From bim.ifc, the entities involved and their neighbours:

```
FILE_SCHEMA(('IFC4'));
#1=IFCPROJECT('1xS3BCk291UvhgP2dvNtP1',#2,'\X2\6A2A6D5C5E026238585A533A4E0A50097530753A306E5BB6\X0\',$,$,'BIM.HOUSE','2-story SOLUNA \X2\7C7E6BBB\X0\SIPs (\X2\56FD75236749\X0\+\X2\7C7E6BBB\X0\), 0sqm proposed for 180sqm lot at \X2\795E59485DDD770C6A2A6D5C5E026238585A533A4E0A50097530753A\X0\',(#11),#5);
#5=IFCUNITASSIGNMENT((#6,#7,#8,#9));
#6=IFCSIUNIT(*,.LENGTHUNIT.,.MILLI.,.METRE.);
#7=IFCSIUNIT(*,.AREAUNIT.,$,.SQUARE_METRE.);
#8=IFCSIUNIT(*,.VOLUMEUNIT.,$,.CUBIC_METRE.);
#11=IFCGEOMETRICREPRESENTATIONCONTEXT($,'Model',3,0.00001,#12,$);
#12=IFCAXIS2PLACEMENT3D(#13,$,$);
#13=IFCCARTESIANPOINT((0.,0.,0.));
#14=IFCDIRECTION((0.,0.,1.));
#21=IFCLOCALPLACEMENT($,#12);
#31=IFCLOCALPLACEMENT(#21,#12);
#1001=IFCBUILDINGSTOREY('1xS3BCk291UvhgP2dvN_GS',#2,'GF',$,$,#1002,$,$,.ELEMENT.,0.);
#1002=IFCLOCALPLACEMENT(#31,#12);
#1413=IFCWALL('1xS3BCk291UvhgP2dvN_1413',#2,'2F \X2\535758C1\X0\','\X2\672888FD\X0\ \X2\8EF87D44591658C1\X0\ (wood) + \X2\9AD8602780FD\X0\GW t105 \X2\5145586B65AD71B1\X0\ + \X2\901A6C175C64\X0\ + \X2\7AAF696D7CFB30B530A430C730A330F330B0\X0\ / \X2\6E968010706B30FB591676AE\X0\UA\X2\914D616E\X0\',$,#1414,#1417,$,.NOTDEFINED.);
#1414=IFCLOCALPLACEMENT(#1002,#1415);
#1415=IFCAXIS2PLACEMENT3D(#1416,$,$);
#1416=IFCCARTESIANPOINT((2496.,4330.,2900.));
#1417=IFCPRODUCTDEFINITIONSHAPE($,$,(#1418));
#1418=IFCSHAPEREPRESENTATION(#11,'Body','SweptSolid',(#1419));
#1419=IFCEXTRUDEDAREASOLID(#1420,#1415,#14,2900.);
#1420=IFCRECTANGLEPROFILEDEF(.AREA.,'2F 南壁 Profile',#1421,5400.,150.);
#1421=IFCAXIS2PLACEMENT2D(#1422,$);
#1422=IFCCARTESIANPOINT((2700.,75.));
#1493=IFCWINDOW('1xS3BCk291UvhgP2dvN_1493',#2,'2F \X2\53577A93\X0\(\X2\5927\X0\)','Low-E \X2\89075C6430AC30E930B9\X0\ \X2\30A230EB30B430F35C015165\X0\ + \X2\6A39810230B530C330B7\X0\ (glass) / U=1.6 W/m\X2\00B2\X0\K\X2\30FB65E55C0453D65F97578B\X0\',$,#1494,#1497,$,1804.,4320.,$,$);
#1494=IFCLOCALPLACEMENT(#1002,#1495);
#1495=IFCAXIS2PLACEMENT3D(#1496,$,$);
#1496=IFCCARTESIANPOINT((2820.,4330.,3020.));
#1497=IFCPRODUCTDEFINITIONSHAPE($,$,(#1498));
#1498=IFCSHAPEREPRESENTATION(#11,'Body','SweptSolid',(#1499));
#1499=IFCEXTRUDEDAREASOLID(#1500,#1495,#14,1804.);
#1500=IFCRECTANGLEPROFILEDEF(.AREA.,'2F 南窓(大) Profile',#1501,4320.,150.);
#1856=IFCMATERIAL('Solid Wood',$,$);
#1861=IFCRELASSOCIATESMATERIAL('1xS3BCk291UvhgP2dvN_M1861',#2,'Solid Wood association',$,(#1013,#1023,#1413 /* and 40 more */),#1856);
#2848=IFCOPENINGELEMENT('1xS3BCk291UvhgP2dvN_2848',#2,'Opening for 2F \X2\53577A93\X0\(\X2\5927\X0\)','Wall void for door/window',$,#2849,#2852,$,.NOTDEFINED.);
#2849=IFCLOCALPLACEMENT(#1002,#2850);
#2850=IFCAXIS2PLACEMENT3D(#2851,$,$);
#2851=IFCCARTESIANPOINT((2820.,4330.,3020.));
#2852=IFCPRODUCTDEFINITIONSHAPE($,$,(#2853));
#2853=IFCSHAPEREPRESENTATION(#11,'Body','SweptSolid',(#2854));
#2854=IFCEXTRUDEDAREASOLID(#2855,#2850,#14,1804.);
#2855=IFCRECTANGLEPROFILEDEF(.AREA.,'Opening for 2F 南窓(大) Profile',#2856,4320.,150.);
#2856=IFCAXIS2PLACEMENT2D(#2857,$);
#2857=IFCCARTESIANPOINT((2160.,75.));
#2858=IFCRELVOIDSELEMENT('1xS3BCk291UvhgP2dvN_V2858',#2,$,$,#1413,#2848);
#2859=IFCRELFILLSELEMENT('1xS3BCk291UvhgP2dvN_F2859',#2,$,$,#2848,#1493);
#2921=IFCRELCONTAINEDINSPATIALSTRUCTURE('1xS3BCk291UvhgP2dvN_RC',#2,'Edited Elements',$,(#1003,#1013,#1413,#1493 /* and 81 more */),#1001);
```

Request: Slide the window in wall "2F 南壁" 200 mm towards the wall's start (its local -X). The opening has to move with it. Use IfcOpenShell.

```python
import ifcopenshell
import ifcopenshell.api.geometry
import ifcopenshell.util.placement

model = ifcopenshell.open("bim.ifc")

window = model.by_guid("1xS3BCk291UvhgP2dvN_1493")
opening = window.FillsVoids[0].RelatingOpeningElement
wall = opening.VoidsElements[0].RelatingBuildingElement

wall_matrix = ifcopenshell.util.placement.get_local_placement(wall.ObjectPlacement)
shift = wall_matrix[:3, 0] * -200.0
before = ifcopenshell.util.placement.get_local_placement(window.ObjectPlacement)[:3, 3].copy()

# The window is not placed relative to its opening, so move both.
for product in (opening, window):
    matrix = ifcopenshell.util.placement.get_local_placement(product.ObjectPlacement)
    matrix[:3, 3] += shift
    ifcopenshell.api.geometry.edit_object_placement(model, product=product, matrix=matrix, is_si=False)

after = ifcopenshell.util.placement.get_local_placement(window.ObjectPlacement)[:3, 3]
print("window moved by", (after - before).round(3) + 0.0)

model.write("bim_updated.ifc")
```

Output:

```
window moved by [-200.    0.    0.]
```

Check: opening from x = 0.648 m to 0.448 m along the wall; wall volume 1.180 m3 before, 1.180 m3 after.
